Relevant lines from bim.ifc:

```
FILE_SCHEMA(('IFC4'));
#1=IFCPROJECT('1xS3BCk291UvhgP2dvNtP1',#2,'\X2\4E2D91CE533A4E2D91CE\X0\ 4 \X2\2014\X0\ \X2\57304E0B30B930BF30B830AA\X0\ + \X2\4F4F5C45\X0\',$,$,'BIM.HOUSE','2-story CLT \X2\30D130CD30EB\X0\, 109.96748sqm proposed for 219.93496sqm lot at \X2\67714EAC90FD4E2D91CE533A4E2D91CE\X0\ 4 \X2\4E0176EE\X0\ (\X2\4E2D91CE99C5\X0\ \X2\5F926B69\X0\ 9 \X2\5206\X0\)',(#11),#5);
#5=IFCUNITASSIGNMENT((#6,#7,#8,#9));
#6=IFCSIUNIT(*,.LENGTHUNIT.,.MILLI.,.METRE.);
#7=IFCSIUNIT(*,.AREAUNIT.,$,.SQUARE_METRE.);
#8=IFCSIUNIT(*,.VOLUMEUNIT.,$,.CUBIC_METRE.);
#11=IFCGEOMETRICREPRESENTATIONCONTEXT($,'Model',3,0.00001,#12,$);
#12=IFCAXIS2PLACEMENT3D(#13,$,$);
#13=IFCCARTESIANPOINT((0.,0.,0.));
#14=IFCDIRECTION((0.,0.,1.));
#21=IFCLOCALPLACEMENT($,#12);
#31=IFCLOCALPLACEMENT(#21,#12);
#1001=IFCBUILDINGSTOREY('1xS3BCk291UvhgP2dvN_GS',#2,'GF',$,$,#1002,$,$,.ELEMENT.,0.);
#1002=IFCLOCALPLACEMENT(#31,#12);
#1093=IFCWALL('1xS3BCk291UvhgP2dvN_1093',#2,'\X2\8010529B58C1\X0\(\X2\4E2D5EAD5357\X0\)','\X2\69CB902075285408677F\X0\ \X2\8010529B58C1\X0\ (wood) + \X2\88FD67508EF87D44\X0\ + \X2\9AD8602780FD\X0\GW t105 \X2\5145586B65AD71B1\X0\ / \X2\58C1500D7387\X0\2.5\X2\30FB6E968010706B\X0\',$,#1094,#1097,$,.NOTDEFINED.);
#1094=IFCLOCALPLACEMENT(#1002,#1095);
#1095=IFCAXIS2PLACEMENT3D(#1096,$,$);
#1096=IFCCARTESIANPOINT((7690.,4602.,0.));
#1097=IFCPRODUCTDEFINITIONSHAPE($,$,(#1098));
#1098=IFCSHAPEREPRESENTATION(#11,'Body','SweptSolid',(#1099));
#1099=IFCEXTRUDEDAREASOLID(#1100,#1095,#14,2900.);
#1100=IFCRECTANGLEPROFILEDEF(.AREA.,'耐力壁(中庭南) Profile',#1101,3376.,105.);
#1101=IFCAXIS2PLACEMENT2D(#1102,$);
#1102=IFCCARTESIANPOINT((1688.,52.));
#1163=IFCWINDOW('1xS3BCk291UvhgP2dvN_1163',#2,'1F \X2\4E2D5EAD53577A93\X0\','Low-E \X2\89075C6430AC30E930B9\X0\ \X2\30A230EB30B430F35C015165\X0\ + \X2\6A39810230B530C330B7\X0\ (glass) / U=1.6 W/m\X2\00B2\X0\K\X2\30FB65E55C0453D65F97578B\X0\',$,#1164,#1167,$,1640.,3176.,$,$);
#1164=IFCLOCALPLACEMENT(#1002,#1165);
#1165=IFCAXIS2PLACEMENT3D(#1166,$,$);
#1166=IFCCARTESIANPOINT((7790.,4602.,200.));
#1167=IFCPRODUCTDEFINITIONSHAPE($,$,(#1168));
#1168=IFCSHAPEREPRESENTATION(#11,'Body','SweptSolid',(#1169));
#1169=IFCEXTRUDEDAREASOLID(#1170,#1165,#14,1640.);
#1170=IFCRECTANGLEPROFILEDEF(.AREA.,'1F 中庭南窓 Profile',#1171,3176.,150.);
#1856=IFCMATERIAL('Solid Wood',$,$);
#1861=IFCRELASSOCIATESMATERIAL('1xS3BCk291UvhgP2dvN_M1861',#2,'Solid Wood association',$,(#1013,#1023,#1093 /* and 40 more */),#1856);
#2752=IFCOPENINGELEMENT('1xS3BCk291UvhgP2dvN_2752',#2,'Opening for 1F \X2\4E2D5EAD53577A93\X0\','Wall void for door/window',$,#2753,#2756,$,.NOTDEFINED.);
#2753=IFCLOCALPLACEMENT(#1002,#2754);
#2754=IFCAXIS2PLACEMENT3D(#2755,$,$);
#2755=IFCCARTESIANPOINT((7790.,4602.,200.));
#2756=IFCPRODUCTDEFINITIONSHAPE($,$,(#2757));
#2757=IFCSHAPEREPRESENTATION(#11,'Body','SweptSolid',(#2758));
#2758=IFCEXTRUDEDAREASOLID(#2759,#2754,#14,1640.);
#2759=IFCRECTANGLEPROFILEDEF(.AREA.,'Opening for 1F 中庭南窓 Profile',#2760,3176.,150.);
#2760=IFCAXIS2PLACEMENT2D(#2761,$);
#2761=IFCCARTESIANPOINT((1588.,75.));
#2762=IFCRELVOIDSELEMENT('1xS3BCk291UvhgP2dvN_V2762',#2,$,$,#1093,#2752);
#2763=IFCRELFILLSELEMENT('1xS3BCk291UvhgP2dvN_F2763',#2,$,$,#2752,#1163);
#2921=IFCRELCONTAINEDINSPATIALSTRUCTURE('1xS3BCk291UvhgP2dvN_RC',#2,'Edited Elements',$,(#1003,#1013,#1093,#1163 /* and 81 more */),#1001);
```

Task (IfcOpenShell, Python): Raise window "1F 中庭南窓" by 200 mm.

```python
import numpy as np
import ifcopenshell
import ifcopenshell.api.geometry
import ifcopenshell.util.placement
import ifcopenshell.util.unit

model = ifcopenshell.open("bim.ifc")
unit_scale = ifcopenshell.util.unit.calculate_unit_scale(model)

window = model.by_guid("1xS3BCk291UvhgP2dvN_1163")
opening = window.FillsVoids[0].RelatingOpeningElement
dz = 200.0

shift = np.array([0.0, 0.0, dz])
# The window is not placed relative to its opening, so move both.
for product in (opening, window):
    matrix = ifcopenshell.util.placement.get_local_placement(product.ObjectPlacement)
    matrix[:3, 3] += shift
    ifcopenshell.api.geometry.edit_object_placement(model, product=product, matrix=matrix, is_si=False)

print(f"moved by {dz * unit_scale:+.3f} m")

model.write("bim_edited.ifc")
```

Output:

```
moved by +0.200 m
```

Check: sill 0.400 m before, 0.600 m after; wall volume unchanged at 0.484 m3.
